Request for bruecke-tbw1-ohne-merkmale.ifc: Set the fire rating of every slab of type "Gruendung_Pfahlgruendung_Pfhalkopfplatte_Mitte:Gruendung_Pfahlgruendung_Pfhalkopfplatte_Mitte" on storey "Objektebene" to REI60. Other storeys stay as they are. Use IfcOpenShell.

First a look at what the model holds.

```python
import ifcopenshell
import ifcopenshell.util.element

model = ifcopenshell.open("bruecke-tbw1-ohne-merkmale.ifc")
print(model.schema)
storey = next(s for s in model.by_type("IfcBuildingStorey") if s.Name == "Objektebene")
slabs = [e for e in ifcopenshell.util.element.get_decomposition(storey) if e.is_a("IfcSlab")]
seen = {}
for e in slabs:
    element_type = ifcopenshell.util.element.get_type(e)
    key = (element_type.Name if element_type != e and element_type else None, ifcopenshell.util.element.get_pset(e, "Pset_SlabCommon", "FireRating"))
    seen[key] = seen.get(key, 0) + 1
for (name, value), count in sorted(seen.items(), key=str):
    print(count, "x", name, "|", value)
```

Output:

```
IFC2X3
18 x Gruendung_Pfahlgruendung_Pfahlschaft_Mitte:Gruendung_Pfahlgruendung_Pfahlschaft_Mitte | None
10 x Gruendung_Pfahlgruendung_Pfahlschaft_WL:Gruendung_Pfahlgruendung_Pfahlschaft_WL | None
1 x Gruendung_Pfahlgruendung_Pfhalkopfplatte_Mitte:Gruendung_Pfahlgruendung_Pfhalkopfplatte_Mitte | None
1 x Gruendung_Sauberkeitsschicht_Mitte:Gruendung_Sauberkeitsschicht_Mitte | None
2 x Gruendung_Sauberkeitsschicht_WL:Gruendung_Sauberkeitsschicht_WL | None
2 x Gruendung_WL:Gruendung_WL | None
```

```python
import ifcopenshell
import ifcopenshell.api.pset
import ifcopenshell.util.element

model = ifcopenshell.open("bruecke-tbw1-ohne-merkmale.ifc")

storey = next(s for s in model.by_type("IfcBuildingStorey") if s.Name == "Objektebene")
slabs = [e for e in ifcopenshell.util.element.get_decomposition(storey) if e.is_a("IfcSlab")]

count = 0
for e in slabs:
    element_type = ifcopenshell.util.element.get_type(e)
    if element_type in (None, e) or element_type.Name != "Gruendung_Pfahlgruendung_Pfhalkopfplatte_Mitte:Gruendung_Pfahlgruendung_Pfhalkopfplatte_Mitte":
        continue
    # add_pset returns the element's existing set when there is one.
    pset = ifcopenshell.api.pset.add_pset(model, product=e, name="Pset_SlabCommon")
    ifcopenshell.api.pset.edit_pset(model, pset=pset, properties={"FireRating": "REI60"})
    count += 1

print(count, "slabs updated")

model.write("bruecke-tbw1-ohne-merkmale_edited.ifc")
```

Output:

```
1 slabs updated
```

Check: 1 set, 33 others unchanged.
